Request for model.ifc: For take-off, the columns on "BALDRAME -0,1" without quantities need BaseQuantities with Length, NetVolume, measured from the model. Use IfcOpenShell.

First a look at what the model holds.

```python
import ifcopenshell
import ifcopenshell.util.element
import ifcopenshell.util.unit

model = ifcopenshell.open("model.ifc")
print(model.schema)
for unit_type in ("LENGTHUNIT", "AREAUNIT", "VOLUMEUNIT"):
    print(unit_type, ifcopenshell.util.unit.calculate_unit_scale(model, unit_type))
storey = next(s for s in model.by_type("IfcBuildingStorey") if s.Name == "BALDRAME -0,1")
columns = [e for e in ifcopenshell.util.element.get_decomposition(storey) if e.is_a("IfcColumn")]
for e in sorted(columns, key=lambda e: e.id()):
    print(e.id(), e.is_a(), e.Name, list(ifcopenshell.util.element.get_psets(e, qtos_only=True)), sep=" | ")
```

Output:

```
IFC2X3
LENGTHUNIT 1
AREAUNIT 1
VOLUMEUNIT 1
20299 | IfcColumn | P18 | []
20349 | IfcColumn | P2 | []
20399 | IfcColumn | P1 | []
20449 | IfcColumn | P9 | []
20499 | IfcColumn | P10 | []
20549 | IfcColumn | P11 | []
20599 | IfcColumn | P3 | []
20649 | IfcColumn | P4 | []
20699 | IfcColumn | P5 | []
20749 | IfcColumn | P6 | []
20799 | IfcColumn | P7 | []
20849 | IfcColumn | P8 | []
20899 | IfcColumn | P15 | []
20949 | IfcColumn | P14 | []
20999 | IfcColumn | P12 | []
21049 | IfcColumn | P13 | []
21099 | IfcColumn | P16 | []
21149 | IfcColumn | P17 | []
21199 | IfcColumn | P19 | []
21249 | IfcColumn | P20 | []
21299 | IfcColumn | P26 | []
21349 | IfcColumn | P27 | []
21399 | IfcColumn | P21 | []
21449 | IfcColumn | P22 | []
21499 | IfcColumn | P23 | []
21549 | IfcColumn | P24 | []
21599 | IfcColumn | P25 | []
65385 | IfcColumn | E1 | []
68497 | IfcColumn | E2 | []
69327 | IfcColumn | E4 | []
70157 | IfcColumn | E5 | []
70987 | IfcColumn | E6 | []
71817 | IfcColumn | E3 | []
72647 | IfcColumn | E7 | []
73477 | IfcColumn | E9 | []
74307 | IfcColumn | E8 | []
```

```python
import ifcopenshell
import ifcopenshell.api.pset
import ifcopenshell.geom
import ifcopenshell.util.element
import ifcopenshell.util.shape
import ifcopenshell.util.unit

model = ifcopenshell.open("model.ifc")
unit_scale = ifcopenshell.util.unit.calculate_unit_scale(model)
volume_scale = ifcopenshell.util.unit.calculate_unit_scale(model, "VOLUMEUNIT")
settings = ifcopenshell.geom.settings()

storey = next(s for s in model.by_type("IfcBuildingStorey") if s.Name == "BALDRAME -0,1")
columns = [e for e in ifcopenshell.util.element.get_decomposition(storey) if e.is_a("IfcColumn")]

for e in sorted(columns, key=lambda e: e.id()):
    if ifcopenshell.util.element.get_psets(e, qtos_only=True, should_inherit=False):
        continue
    # Geometry comes back in metres, in the element's own axes.
    shape = ifcopenshell.geom.create_shape(settings, e)
    values = {
        "Length": ifcopenshell.util.shape.get_z(shape.geometry) / unit_scale,
        "NetVolume": ifcopenshell.util.shape.get_volume(shape.geometry) / volume_scale,
    }
    qto = ifcopenshell.api.pset.add_qto(model, product=e, name="BaseQuantities")
    ifcopenshell.api.pset.edit_qto(model, qto=qto, properties=values)
    print(e.id(), {k: round(v, 3) for k, v in values.items()})

model.write("model_edited.ifc")
```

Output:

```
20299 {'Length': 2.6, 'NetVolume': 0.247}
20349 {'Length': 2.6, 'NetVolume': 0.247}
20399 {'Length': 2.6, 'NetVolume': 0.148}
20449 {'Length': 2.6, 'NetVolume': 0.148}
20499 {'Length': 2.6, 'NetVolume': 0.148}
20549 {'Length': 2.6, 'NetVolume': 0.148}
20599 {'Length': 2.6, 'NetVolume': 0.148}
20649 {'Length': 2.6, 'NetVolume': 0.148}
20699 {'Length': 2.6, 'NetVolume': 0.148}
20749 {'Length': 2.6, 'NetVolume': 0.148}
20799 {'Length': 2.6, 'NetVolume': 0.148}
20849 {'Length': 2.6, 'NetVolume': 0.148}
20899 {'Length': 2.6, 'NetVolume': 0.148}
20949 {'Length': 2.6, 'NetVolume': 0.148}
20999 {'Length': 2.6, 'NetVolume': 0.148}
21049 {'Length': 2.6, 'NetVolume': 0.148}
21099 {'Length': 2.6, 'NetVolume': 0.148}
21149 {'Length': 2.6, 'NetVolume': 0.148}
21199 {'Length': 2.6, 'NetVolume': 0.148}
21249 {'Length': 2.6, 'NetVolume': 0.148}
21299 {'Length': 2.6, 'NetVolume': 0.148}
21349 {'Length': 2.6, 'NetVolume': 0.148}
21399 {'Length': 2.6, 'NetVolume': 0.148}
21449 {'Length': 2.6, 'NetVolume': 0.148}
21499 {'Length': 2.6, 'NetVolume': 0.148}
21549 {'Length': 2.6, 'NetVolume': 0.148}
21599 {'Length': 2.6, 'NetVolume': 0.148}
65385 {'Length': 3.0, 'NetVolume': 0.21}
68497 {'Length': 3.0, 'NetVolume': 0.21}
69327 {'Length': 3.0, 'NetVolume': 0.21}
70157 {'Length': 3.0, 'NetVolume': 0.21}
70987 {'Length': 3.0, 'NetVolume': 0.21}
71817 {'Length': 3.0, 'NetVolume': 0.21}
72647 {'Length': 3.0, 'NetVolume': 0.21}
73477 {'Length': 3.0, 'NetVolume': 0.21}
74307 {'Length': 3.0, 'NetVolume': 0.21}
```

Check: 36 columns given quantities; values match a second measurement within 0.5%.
